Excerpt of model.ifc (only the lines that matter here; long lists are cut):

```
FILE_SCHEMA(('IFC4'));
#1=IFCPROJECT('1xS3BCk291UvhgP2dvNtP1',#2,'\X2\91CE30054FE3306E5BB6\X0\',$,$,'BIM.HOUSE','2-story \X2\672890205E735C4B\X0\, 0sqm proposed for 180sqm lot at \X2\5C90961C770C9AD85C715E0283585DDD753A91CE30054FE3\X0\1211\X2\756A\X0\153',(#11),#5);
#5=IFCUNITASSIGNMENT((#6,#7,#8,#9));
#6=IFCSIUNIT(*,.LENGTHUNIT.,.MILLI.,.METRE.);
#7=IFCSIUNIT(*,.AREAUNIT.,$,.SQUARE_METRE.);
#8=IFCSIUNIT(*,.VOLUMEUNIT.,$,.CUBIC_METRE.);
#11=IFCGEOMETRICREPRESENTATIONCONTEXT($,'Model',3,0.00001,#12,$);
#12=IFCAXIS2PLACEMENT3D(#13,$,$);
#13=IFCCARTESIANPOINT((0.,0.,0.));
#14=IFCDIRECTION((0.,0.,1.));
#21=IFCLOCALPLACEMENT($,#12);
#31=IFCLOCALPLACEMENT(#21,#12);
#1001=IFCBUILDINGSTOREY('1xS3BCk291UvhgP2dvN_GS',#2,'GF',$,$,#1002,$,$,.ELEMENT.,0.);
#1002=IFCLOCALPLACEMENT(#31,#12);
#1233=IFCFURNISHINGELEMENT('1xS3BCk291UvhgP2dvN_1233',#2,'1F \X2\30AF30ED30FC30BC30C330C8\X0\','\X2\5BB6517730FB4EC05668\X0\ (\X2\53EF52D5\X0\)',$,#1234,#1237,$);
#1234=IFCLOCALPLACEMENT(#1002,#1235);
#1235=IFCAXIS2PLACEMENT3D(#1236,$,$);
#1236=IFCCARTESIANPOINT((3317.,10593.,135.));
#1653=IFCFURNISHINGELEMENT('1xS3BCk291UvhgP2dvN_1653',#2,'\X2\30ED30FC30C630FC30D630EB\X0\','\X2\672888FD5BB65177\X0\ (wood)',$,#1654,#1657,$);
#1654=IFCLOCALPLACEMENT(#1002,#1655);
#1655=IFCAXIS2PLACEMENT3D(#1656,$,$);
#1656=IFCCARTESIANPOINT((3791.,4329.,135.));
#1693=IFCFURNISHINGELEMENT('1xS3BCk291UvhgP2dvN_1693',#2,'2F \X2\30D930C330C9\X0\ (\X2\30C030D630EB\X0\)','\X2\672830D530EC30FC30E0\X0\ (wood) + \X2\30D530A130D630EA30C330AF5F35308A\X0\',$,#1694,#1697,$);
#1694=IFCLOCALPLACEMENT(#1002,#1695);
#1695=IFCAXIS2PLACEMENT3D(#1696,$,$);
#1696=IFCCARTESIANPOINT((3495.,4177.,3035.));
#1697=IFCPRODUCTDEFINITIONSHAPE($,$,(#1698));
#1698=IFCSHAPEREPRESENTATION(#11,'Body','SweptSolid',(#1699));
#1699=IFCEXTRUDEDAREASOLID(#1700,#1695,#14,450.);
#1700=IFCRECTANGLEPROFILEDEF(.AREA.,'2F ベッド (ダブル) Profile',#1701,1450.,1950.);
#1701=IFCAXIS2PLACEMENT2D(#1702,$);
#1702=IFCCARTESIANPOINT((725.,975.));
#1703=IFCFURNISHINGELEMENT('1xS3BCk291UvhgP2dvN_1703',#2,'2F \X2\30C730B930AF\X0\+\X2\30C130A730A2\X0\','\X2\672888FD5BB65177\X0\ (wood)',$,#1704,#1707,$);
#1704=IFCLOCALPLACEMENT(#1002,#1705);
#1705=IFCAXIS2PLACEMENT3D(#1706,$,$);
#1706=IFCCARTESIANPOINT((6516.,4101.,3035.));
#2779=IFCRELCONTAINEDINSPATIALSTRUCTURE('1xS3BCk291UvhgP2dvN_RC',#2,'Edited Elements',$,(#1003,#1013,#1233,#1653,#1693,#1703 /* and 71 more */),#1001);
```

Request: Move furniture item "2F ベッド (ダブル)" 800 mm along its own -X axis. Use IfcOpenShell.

```python
import ifcopenshell
import ifcopenshell.api.geometry
import ifcopenshell.util.placement
import ifcopenshell.util.unit

model = ifcopenshell.open("model.ifc")
unit_scale = ifcopenshell.util.unit.calculate_unit_scale(model)

item = model.by_guid("1xS3BCk291UvhgP2dvN_1693")
matrix = ifcopenshell.util.placement.get_local_placement(item.ObjectPlacement)
matrix[:3, 3] -= matrix[:3, 0] * 0.8 / unit_scale
ifcopenshell.api.geometry.edit_object_placement(model, product=item, matrix=matrix, is_si=False)

print(ifcopenshell.util.placement.get_local_placement(item.ObjectPlacement).round(3) + 0.0)

model.write("model-out.ifc")
```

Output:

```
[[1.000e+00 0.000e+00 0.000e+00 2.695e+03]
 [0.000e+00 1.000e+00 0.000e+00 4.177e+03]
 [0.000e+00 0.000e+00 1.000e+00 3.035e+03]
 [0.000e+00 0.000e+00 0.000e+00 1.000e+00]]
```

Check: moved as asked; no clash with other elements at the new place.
